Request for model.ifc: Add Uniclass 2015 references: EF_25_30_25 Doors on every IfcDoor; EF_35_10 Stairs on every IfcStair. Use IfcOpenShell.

First a look at what the model holds.

```python
import ifcopenshell

model = ifcopenshell.open("model.ifc")
print(model.schema)
print("classifications:", [c.Name for c in model.by_type("IfcClassification")])
for ifc_class in ("IfcDoor", "IfcRoof", "IfcStair", "IfcWall", "IfcWindow"):
    print(ifc_class, len(model.by_type(ifc_class)))
```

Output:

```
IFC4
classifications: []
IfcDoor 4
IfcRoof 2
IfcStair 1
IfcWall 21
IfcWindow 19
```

```python
import ifcopenshell
import ifcopenshell.api.classification

model = ifcopenshell.open("model.ifc")

system = ifcopenshell.api.classification.add_classification(model, classification="Uniclass 2015")

codes = {
    "IfcDoor": ("EF_25_30_25", "Doors"),
    "IfcStair": ("EF_35_10", "Stairs"),
}
for ifc_class, (code, name) in codes.items():
    products = model.by_type(ifc_class)
    ifcopenshell.api.classification.add_reference(
        model, products=products, classification=system, identification=code, name=name
    )
    print(code, len(products))

model.write("model_edited.ifc")
```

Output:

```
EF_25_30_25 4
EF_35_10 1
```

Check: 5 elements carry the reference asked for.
